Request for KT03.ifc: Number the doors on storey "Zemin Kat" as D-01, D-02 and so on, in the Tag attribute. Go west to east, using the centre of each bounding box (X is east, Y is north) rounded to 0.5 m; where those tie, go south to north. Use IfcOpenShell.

First a look at what the model holds.

```python
import ifcopenshell
import ifcopenshell.util.element
import ifcopenshell.util.placement

model = ifcopenshell.open("KT03.ifc")
print(model.schema)
storey = next(s for s in model.by_type("IfcBuildingStorey") if s.Name == "Zemin Kat")
doors = [e for e in ifcopenshell.util.element.get_decomposition(storey) if e.is_a("IfcDoor")]
for e in sorted(doors, key=lambda e: e.id()):
    origin = ifcopenshell.util.placement.get_local_placement(e.ObjectPlacement)[:3, 3]
    print(e.id(), e.Tag, e.Name, origin.round(2) + 0.0, sep=" | ")
```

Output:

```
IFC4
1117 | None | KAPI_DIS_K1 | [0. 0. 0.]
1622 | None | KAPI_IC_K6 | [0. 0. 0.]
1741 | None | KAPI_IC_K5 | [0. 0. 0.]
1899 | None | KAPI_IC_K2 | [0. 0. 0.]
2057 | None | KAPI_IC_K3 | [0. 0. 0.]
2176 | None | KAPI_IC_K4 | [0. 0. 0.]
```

```python
import ifcopenshell
import ifcopenshell.geom
import ifcopenshell.util.element
import ifcopenshell.util.shape

model = ifcopenshell.open("KT03.ifc")
settings = ifcopenshell.geom.settings()
settings.set("use-world-coords", True)


def centre(element):
    shape = ifcopenshell.geom.create_shape(settings, element)
    return ifcopenshell.util.shape.get_bbox_centroid(shape.geometry)


storey = next(s for s in model.by_type("IfcBuildingStorey") if s.Name == "Zemin Kat")
doors = [e for e in ifcopenshell.util.element.get_decomposition(storey) if e.is_a("IfcDoor")]

# Insertion points can sit at a corner or the storey origin, so sort by the geometry (in metres).
centres = {e: centre(e) for e in doors}
doors.sort(key=lambda e: (round(centres[e][0] / 0.5), centres[e][1]))

for i, e in enumerate(doors, start=1):
    number = f"D-{i:02d}"
    e.Tag = number
    print(e.id(), number)

model.write("KT03_v2.ifc")
```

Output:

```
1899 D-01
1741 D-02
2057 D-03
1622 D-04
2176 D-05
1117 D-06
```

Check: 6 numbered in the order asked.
